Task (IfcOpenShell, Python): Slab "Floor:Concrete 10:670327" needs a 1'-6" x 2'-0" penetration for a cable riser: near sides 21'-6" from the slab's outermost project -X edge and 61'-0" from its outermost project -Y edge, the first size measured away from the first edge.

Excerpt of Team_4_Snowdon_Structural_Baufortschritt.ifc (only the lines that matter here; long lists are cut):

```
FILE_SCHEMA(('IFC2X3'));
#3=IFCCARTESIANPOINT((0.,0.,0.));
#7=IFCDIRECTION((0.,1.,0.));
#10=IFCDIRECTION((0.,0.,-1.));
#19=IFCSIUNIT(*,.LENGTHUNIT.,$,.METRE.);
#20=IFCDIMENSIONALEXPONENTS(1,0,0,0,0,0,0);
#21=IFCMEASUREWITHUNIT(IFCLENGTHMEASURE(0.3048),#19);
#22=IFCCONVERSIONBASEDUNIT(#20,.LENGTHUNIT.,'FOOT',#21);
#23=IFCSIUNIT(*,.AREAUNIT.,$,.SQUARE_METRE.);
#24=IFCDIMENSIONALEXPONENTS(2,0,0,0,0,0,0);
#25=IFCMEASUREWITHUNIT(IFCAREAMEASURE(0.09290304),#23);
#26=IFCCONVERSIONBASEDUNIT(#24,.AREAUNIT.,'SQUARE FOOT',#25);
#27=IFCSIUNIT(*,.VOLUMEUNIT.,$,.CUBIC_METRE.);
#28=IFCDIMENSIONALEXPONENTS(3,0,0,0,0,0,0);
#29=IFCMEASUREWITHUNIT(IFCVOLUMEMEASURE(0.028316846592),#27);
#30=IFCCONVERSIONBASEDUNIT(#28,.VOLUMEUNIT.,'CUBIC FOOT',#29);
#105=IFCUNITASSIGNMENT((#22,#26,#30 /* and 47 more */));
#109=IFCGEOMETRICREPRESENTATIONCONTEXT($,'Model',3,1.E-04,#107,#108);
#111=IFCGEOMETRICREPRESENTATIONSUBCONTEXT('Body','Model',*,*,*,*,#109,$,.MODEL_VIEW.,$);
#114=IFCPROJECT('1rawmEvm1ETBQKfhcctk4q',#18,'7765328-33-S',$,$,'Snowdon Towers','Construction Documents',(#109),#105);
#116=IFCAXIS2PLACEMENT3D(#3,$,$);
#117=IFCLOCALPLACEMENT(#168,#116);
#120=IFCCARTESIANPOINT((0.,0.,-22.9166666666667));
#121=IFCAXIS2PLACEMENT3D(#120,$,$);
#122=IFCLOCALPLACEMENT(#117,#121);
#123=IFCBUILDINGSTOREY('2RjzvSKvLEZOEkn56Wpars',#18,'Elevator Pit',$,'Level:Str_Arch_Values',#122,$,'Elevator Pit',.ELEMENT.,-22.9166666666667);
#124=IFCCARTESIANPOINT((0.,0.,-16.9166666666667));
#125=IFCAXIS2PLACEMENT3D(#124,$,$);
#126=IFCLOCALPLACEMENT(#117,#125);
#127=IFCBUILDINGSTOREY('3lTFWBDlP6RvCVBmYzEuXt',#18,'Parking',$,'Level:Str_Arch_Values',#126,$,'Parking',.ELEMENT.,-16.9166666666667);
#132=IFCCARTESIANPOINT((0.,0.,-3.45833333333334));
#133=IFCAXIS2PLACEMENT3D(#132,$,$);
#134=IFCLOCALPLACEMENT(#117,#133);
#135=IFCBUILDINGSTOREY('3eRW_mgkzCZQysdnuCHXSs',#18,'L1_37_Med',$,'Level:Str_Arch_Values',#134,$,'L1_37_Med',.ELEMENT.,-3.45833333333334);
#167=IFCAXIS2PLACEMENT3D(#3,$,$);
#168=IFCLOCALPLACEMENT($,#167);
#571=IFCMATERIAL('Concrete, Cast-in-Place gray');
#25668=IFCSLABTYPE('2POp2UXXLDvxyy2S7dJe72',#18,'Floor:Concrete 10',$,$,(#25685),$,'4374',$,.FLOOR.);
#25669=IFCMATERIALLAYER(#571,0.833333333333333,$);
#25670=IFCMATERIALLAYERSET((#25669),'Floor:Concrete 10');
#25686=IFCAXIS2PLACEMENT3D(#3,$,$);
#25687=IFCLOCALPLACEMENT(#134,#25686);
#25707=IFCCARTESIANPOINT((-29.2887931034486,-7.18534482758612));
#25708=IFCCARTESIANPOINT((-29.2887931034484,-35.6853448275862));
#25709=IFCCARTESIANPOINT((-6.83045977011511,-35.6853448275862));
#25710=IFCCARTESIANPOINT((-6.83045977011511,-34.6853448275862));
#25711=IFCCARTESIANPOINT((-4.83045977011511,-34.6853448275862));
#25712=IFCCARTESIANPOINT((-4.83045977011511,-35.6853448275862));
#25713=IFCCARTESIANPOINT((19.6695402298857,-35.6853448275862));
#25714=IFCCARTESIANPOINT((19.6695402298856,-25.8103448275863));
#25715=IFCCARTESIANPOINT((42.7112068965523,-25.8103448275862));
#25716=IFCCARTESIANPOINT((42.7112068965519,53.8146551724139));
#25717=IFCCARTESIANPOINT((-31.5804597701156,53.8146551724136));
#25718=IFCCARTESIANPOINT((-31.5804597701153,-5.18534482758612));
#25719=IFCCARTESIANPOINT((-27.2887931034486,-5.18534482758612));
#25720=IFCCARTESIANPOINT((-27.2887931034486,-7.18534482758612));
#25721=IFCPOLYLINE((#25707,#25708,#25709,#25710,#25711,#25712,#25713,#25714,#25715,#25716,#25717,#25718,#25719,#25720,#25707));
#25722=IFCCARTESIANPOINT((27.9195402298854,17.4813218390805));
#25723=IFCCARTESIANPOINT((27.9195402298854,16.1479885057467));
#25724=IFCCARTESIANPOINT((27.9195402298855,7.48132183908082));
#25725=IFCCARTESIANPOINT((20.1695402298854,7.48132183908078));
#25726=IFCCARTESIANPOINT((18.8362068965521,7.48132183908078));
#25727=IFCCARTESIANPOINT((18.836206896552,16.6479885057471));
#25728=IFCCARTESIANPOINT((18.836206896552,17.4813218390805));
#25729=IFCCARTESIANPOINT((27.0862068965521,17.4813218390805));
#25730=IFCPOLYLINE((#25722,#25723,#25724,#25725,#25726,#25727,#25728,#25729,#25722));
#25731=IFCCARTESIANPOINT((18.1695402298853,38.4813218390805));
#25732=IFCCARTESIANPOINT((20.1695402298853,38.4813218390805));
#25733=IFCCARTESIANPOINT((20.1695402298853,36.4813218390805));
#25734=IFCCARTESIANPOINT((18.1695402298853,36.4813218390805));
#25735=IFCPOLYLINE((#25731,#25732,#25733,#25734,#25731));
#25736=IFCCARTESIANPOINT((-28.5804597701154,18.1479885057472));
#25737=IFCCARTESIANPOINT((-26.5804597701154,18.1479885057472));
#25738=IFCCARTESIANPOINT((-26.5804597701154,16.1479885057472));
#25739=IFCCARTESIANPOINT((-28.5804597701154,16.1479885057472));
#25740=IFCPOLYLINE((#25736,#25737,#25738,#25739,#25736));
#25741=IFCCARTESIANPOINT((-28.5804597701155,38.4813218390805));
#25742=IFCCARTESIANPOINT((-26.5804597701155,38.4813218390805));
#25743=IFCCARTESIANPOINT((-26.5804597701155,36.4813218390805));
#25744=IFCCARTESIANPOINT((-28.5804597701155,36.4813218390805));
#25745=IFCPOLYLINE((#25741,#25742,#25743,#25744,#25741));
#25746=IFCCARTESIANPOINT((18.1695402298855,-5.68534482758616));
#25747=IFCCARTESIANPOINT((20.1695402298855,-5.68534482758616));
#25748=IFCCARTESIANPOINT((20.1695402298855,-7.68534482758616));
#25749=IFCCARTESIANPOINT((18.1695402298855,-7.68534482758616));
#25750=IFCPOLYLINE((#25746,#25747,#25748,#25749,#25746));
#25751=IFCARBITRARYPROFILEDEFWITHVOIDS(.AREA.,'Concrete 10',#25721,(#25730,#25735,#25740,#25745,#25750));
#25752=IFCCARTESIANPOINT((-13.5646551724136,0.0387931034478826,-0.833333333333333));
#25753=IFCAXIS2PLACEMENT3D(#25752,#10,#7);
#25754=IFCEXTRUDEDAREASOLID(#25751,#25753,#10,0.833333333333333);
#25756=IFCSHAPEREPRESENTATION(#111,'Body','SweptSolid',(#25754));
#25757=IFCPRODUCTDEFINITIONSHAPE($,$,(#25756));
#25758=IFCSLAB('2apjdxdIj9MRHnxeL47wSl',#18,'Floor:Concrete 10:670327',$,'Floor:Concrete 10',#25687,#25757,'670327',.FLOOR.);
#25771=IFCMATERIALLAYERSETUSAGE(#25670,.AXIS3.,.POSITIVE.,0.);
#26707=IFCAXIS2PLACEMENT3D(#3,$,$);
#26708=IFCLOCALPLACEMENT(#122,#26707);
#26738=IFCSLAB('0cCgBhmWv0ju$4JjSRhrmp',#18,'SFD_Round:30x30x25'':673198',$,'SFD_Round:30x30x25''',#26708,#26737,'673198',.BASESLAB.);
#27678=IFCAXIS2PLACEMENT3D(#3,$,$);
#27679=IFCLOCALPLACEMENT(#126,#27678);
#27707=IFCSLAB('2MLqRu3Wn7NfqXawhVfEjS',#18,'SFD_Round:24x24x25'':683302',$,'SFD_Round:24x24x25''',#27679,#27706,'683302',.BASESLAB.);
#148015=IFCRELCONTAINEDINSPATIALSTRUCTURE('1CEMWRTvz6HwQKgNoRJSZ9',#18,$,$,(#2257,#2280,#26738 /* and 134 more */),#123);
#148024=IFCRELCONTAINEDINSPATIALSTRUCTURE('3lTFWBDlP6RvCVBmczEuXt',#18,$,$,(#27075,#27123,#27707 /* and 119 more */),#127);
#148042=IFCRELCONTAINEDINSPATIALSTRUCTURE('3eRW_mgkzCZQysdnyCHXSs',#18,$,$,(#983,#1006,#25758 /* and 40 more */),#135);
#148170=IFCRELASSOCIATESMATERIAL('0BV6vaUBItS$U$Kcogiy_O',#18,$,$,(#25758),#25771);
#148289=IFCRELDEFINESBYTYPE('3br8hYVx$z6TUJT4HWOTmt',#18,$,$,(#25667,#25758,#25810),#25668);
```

```python
import numpy as np
import ifcopenshell
import ifcopenshell.api.feature
import ifcopenshell.api.geometry
import ifcopenshell.api.root
import ifcopenshell.geom
import ifcopenshell.util.placement
import ifcopenshell.util.representation
import ifcopenshell.util.shape
import ifcopenshell.util.unit

model = ifcopenshell.open("Team_4_Snowdon_Structural_Baufortschritt.ifc")
unit_scale = ifcopenshell.util.unit.calculate_unit_scale(model)
settings = ifcopenshell.geom.settings()


def volume(element):
    """Net volume in cubic metres, openings subtracted."""
    shape = ifcopenshell.geom.create_shape(settings, element)
    return ifcopenshell.util.shape.get_volume(shape.geometry)


slab = model.by_id(25758)
before = volume(slab)

# Extent in the slab's own axes, in metres. The edges named are its -X and -Y sides.
slab_shape = ifcopenshell.geom.create_shape(settings, slab)
vertices = ifcopenshell.util.shape.get_vertices(slab_shape.geometry)
x_min, y_min, bottom = vertices.min(axis=0)
top = vertices[:, 2].max()

opening = ifcopenshell.api.root.create_entity(model, ifc_class="IfcOpeningElement", name="Cable riser opening")
context = ifcopenshell.util.representation.get_context(model, "Model", "Body", "MODEL_VIEW")
width, depth = 0.4572, 0.6096
outline = [(0.0, 0.0), (width, 0.0), (width, depth), (0.0, depth), (0.0, 0.0)]
# Overshoot both faces by 50 mm so the cut is clean.
shape = ifcopenshell.api.geometry.add_slab_representation(
    model, context=context, depth=top - bottom + 0.1, polyline=outline
)
ifcopenshell.api.geometry.assign_representation(model, product=opening, representation=shape)

matrix = ifcopenshell.util.placement.get_local_placement(slab.ObjectPlacement)
matrix[:, 3] = matrix @ np.append(np.array([x_min + 6.5532, y_min + 18.5928, bottom - 0.05]) / unit_scale, 1.0)
ifcopenshell.api.geometry.edit_object_placement(model, product=opening, matrix=matrix, is_si=False)
ifcopenshell.api.feature.add_feature(model, feature=opening, element=slab)

after = volume(slab)

print(f"slab volume {before:.3f} -> {after:.3f} m3")

model.write("Team_4_Snowdon_Structural_Baufortschritt_updated.ifc")
```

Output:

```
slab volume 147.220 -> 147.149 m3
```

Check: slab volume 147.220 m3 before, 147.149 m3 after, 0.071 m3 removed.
